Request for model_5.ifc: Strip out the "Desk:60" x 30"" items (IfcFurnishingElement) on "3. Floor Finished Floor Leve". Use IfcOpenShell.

First a look at what the model holds.

```python
import ifcopenshell
import ifcopenshell.util.element

model = ifcopenshell.open("model_5.ifc")
print(model.schema)
storey = next(s for s in model.by_type("IfcBuildingStorey") if s.Name == "3. Floor Finished Floor Leve")
furniture = [e for e in ifcopenshell.util.element.get_decomposition(storey) if e.is_a("IfcFurnishingElement")]
seen = {}
for e in furniture:
    element_type = ifcopenshell.util.element.get_type(e)
    name = element_type.Name if element_type not in (None, e) else None
    seen[name] = seen.get(name, 0) + 1
for name, count in sorted(seen.items(), key=str):
    print(count, "x", name)
```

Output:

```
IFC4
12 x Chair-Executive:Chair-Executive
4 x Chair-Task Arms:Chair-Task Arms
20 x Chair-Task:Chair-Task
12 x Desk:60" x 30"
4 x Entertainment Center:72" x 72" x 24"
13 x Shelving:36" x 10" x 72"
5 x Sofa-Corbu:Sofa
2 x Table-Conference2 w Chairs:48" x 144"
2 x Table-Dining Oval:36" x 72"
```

```python
import ifcopenshell
import ifcopenshell.api.root
import ifcopenshell.util.element

model = ifcopenshell.open("model_5.ifc")

storey = next(s for s in model.by_type("IfcBuildingStorey") if s.Name == "3. Floor Finished Floor Leve")
furniture = [e for e in ifcopenshell.util.element.get_decomposition(storey) if e.is_a("IfcFurnishingElement")]
targets = [e for e in furniture if (t := ifcopenshell.util.element.get_type(e)) not in (None, e) and t.Name == 'Desk:60" x 30"']

for e in targets:
    ifcopenshell.api.root.remove_product(model, product=e)
print(len(targets), "removed")

model.write("model_5-out.ifc")
```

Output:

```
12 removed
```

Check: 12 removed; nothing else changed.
